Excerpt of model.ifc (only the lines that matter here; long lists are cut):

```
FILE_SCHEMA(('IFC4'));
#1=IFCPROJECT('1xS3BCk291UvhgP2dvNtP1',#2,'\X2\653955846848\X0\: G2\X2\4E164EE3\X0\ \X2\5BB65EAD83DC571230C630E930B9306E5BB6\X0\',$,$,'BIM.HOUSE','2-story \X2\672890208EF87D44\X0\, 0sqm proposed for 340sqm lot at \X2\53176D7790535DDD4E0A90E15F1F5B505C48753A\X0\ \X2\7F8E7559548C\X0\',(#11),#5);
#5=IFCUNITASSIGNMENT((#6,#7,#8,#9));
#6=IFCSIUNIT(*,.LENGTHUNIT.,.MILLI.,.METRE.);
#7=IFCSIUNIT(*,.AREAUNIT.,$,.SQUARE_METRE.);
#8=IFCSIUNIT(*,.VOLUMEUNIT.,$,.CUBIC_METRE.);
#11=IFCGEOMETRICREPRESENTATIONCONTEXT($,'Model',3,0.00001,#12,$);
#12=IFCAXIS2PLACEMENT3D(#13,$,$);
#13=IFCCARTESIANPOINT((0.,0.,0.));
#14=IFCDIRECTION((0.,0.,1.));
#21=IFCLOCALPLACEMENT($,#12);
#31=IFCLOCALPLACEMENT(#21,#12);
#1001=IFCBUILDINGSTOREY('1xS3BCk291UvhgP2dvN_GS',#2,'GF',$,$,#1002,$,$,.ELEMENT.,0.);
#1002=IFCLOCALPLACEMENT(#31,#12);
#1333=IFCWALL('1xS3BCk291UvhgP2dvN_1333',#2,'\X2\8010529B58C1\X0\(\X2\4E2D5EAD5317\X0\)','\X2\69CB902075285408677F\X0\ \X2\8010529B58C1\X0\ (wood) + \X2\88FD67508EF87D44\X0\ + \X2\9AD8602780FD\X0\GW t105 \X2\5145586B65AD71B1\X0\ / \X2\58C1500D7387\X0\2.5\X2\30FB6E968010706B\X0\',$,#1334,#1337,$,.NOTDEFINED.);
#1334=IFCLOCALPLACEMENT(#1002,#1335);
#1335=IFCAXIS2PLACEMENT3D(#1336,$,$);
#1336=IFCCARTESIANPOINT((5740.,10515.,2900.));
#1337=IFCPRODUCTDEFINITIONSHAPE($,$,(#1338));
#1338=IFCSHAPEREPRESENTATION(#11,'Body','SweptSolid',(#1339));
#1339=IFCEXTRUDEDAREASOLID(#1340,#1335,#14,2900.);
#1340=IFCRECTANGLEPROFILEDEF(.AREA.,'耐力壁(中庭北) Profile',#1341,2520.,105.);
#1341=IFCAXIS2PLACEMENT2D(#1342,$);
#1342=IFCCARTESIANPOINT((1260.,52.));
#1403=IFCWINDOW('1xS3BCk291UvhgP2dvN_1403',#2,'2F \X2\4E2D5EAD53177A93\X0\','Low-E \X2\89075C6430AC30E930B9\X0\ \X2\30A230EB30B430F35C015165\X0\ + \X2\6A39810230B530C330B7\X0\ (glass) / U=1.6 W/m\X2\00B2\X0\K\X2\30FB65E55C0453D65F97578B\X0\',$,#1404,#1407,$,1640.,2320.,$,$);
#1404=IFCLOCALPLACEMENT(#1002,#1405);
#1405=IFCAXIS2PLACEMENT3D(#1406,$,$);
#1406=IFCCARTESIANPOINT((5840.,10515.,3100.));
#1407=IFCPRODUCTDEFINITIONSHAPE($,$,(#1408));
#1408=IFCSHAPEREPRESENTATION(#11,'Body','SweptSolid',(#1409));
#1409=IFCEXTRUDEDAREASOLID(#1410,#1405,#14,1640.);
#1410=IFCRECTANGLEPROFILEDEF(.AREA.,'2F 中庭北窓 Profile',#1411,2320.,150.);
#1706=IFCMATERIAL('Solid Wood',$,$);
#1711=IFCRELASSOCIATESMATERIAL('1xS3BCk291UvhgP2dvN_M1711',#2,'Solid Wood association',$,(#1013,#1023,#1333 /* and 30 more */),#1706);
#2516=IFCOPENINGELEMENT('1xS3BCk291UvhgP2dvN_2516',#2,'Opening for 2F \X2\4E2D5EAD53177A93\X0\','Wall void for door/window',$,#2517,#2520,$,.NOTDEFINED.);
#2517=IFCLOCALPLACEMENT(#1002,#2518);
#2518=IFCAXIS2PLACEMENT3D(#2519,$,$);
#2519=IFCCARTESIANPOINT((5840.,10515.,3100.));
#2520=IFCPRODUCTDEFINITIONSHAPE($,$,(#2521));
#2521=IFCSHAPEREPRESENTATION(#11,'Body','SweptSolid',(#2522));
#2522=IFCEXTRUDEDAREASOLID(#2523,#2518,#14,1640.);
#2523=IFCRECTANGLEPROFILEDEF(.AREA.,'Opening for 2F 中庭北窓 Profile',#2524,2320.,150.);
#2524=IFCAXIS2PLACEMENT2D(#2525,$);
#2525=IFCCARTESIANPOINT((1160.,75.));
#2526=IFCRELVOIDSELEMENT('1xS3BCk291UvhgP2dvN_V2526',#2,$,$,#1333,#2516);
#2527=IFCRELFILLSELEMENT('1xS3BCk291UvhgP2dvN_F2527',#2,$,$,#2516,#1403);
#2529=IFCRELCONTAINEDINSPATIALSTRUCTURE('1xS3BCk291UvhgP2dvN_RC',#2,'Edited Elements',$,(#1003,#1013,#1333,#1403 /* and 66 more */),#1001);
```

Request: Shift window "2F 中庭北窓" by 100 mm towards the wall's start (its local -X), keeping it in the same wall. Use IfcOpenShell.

```python
import ifcopenshell
import ifcopenshell.api.geometry
import ifcopenshell.util.placement
import ifcopenshell.util.unit

model = ifcopenshell.open("model.ifc")
unit_scale = ifcopenshell.util.unit.calculate_unit_scale(model)

window = model.by_id(1403)
opening = window.FillsVoids[0].RelatingOpeningElement
wall = opening.VoidsElements[0].RelatingBuildingElement

wall_matrix = ifcopenshell.util.placement.get_local_placement(wall.ObjectPlacement)
shift = wall_matrix[:3, 0] * -0.1 / unit_scale
before = ifcopenshell.util.placement.get_local_placement(window.ObjectPlacement)[:3, 3].copy()

# The window is not placed relative to its opening, so move both.
for product in (opening, window):
    matrix = ifcopenshell.util.placement.get_local_placement(product.ObjectPlacement)
    matrix[:3, 3] += shift
    ifcopenshell.api.geometry.edit_object_placement(model, product=product, matrix=matrix, is_si=False)

after = ifcopenshell.util.placement.get_local_placement(window.ObjectPlacement)[:3, 3]
print("window moved by", (after - before).round(3) + 0.0)

model.write("model_rev.ifc")
```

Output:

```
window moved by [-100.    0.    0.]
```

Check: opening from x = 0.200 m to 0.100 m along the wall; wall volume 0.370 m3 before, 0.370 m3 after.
